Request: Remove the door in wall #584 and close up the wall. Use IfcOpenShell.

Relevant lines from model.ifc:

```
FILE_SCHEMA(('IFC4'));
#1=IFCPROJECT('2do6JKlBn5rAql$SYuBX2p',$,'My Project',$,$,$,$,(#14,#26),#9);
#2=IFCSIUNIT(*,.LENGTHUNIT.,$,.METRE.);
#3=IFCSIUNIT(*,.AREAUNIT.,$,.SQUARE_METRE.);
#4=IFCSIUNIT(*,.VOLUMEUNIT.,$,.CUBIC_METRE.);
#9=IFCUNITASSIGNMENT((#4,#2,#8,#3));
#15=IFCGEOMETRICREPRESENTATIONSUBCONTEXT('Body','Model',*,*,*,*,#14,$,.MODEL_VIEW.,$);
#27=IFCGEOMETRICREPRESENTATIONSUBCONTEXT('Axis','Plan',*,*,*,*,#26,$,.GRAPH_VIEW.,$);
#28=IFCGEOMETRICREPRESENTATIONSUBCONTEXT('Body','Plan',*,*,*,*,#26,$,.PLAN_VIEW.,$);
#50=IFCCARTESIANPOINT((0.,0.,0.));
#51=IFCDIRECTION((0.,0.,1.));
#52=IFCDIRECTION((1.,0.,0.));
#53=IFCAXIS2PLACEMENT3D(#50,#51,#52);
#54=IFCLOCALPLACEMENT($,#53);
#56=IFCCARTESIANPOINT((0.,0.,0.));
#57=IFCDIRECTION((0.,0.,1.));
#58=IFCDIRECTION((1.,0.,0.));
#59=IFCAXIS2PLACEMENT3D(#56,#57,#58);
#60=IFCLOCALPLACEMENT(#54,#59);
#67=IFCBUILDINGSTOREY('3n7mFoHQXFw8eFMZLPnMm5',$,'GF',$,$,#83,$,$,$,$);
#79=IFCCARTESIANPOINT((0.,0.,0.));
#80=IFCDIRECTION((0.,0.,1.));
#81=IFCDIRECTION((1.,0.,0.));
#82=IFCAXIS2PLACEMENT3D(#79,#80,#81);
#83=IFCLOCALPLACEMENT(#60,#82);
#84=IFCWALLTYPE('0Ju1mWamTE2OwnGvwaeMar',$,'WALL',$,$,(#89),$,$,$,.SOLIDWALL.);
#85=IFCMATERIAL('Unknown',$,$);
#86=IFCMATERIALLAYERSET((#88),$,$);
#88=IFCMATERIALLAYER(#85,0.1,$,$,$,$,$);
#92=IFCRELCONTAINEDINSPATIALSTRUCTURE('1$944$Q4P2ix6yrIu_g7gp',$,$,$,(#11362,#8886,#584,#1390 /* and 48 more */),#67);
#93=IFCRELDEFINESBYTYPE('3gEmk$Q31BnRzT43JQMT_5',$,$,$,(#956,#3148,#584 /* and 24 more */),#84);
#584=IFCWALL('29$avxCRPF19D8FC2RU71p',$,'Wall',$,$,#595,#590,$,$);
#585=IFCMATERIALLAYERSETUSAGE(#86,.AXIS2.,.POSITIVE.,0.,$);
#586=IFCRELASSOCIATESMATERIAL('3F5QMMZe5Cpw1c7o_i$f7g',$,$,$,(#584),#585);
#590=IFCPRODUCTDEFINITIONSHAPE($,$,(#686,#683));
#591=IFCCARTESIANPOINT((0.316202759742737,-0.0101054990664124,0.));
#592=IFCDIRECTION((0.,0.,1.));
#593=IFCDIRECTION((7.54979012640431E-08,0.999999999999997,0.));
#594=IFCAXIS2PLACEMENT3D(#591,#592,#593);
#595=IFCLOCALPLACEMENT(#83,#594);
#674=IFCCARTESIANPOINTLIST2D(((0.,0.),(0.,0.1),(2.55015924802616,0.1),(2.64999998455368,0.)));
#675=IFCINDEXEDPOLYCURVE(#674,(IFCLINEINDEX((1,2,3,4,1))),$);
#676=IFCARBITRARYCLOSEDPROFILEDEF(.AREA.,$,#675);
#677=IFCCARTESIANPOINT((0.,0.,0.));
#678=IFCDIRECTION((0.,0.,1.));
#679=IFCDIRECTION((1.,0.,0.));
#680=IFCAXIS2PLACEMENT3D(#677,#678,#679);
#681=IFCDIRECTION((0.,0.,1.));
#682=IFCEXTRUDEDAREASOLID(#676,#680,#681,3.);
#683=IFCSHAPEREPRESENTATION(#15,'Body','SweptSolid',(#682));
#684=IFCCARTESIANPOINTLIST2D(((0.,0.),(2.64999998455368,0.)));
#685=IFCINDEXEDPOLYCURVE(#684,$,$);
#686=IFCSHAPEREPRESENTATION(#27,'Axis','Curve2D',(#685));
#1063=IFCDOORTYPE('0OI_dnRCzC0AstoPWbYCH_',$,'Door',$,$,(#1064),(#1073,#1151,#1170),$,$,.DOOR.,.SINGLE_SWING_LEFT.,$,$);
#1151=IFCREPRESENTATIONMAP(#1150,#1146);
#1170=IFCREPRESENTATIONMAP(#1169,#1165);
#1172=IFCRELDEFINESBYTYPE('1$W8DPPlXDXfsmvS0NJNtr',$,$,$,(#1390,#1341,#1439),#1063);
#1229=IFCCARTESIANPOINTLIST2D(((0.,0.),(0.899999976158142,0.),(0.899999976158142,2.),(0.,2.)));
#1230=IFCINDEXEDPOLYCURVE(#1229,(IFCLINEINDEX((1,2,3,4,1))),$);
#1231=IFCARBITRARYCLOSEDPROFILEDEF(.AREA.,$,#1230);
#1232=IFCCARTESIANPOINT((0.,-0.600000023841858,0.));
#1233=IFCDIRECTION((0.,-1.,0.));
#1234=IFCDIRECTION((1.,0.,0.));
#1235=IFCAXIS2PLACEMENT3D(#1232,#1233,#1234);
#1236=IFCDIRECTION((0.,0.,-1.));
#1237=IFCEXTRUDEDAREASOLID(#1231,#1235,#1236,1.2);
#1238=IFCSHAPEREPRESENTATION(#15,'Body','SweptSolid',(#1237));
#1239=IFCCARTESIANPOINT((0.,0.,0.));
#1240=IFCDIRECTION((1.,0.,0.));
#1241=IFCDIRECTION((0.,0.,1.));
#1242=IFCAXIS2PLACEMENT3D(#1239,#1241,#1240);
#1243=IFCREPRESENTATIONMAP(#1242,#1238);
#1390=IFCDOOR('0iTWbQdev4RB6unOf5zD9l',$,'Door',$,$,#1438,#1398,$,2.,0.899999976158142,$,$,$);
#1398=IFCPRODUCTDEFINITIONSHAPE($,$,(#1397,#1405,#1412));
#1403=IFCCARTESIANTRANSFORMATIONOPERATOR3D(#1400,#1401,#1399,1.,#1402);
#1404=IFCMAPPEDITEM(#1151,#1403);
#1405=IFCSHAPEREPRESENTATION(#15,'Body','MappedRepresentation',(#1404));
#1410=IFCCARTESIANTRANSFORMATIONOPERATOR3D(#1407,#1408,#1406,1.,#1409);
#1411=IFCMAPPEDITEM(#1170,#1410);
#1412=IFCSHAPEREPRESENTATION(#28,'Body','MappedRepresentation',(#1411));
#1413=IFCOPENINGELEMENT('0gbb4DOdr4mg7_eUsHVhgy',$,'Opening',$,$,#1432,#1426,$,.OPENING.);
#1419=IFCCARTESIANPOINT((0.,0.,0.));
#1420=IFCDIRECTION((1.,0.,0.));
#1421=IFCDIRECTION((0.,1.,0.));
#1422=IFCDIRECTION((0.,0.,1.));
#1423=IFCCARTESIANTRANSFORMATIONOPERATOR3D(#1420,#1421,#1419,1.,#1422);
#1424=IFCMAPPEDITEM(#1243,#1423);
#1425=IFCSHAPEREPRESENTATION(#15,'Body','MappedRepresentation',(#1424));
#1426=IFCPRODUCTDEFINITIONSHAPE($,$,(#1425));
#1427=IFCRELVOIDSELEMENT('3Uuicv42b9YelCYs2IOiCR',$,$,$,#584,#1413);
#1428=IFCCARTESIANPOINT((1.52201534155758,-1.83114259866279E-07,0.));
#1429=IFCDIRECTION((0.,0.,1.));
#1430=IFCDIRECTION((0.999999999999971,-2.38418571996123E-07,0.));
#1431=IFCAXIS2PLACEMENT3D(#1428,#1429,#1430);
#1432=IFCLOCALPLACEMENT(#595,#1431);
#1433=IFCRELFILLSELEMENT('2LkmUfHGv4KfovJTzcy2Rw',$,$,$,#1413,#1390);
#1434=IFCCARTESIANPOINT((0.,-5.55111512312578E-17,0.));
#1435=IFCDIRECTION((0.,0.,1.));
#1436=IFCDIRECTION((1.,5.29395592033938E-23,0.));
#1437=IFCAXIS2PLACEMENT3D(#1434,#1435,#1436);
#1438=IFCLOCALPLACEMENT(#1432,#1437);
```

```python
import ifcopenshell
import ifcopenshell.api.feature
import ifcopenshell.api.root
import ifcopenshell.geom
import ifcopenshell.util.shape

model = ifcopenshell.open("model.ifc")
settings = ifcopenshell.geom.settings()


def volume(element):
    """Net volume in cubic metres, openings subtracted."""
    shape = ifcopenshell.geom.create_shape(settings, element)
    return ifcopenshell.util.shape.get_volume(shape.geometry)


door = model.by_guid("0iTWbQdev4RB6unOf5zD9l")
opening = door.FillsVoids[0].RelatingOpeningElement
wall = opening.VoidsElements[0].RelatingBuildingElement
before = volume(wall)

ifcopenshell.api.root.remove_product(model, product=door)
ifcopenshell.api.feature.remove_feature(model, feature=opening)

after = volume(wall)

print(f"wall volume {before:.3f} -> {after:.3f} m3")

model.write("model_edited.ifc")
```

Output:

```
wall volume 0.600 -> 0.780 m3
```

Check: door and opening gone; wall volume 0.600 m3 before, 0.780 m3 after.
